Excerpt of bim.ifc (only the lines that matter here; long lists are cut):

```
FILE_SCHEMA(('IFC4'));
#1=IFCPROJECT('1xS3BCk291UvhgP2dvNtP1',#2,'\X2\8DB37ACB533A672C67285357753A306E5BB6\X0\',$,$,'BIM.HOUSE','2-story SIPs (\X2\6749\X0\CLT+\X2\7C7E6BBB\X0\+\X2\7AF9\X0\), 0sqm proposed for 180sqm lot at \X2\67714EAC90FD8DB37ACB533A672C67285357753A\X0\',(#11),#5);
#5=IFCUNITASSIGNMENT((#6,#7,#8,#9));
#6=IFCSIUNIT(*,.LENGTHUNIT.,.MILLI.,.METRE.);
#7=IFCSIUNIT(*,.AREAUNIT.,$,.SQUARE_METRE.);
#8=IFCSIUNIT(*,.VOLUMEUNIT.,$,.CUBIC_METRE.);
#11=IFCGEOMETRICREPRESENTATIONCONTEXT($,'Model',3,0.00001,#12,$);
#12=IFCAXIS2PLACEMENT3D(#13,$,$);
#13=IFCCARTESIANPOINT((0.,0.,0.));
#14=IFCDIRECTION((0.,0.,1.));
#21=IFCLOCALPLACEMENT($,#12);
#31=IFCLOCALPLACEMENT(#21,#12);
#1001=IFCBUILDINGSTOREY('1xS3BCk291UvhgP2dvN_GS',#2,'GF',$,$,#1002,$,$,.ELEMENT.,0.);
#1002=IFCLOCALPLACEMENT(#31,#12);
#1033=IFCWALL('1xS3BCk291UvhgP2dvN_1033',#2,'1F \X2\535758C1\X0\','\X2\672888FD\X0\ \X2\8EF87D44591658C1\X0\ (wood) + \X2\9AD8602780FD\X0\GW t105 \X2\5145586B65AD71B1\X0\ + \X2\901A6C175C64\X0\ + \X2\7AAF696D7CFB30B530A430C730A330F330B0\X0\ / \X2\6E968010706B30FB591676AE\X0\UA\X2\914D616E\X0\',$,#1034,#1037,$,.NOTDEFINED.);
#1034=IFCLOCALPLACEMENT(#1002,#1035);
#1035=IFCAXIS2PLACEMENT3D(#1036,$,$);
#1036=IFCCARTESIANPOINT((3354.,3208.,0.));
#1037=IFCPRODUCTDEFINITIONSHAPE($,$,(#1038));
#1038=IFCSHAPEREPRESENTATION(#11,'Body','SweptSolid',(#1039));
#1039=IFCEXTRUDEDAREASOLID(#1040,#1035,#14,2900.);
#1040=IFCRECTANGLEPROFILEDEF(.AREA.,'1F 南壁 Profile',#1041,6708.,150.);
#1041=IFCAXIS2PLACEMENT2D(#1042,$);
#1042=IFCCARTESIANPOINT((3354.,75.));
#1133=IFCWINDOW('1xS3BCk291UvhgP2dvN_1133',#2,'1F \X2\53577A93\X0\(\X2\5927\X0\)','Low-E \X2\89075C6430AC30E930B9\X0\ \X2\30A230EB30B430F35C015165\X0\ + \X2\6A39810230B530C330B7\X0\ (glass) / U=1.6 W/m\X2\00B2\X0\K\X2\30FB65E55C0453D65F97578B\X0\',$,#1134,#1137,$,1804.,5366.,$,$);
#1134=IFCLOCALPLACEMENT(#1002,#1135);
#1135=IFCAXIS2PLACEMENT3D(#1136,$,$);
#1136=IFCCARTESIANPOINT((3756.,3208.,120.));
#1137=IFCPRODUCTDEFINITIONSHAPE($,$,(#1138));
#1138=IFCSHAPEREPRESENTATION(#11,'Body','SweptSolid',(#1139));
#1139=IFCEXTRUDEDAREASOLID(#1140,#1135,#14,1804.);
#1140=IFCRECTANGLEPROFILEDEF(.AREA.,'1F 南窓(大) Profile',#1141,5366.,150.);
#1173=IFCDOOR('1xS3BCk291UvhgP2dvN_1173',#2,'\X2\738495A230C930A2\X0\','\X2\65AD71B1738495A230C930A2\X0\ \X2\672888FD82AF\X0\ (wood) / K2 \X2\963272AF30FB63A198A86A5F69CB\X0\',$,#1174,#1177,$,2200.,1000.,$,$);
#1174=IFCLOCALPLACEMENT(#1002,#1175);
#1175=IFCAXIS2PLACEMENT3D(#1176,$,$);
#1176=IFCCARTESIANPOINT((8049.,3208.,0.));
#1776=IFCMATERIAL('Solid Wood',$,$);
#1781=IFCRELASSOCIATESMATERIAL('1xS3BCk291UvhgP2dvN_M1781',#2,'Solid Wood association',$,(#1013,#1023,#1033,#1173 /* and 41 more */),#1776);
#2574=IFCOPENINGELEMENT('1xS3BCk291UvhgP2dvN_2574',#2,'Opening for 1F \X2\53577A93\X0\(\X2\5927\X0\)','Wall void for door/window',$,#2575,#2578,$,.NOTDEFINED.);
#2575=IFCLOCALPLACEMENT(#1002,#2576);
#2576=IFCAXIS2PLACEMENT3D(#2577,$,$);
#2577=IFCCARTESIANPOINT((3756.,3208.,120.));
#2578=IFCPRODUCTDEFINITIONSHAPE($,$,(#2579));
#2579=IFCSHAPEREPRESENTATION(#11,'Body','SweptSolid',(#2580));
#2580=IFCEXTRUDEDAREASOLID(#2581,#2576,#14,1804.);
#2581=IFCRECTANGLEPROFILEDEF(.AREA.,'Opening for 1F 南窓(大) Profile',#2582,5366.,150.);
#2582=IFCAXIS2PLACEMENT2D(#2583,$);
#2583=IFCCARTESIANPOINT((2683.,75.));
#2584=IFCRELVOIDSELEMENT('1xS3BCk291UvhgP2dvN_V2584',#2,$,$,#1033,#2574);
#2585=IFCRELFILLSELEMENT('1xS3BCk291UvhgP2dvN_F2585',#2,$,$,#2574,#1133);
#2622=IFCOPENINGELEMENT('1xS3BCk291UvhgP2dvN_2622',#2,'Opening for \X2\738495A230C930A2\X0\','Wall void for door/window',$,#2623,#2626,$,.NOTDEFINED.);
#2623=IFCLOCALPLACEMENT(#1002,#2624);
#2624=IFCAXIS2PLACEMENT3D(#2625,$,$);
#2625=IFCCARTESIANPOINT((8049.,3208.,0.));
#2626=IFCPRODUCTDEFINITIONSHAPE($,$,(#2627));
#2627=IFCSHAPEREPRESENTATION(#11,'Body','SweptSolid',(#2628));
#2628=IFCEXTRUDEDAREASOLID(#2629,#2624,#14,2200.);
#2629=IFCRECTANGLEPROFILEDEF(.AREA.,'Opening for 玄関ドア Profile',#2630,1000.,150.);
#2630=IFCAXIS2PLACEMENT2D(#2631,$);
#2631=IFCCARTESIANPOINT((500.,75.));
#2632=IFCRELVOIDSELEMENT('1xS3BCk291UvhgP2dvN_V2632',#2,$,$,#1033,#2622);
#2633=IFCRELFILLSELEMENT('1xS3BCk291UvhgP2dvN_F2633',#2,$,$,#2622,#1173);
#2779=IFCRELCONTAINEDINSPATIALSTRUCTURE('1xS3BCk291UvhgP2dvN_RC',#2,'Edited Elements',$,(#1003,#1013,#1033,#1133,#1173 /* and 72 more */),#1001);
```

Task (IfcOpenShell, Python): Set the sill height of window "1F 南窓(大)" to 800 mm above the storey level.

```python
import numpy as np
import ifcopenshell
import ifcopenshell.api.geometry
import ifcopenshell.geom
import ifcopenshell.util.element
import ifcopenshell.util.placement
import ifcopenshell.util.shape
import ifcopenshell.util.unit

model = ifcopenshell.open("bim.ifc")
unit_scale = ifcopenshell.util.unit.calculate_unit_scale(model)

window = model.by_guid("1xS3BCk291UvhgP2dvN_1133")
opening = window.FillsVoids[0].RelatingOpeningElement
storey = ifcopenshell.util.element.get_container(window, ifc_class="IfcBuildingStorey")
level = ifcopenshell.util.placement.get_local_placement(storey.ObjectPlacement)[2, 3]

# The opening's origin need not be at the sill, so measure its lowest point.
shape = ifcopenshell.geom.create_shape(ifcopenshell.geom.settings(), opening)
bottom = ifcopenshell.util.shape.get_shape_bottom_elevation(shape, shape.geometry) / unit_scale
dz = level + 0.8 / unit_scale - bottom

shift = np.array([0.0, 0.0, dz])
# The window is not placed relative to its opening, so move both.
for product in (opening, window):
    matrix = ifcopenshell.util.placement.get_local_placement(product.ObjectPlacement)
    matrix[:3, 3] += shift
    ifcopenshell.api.geometry.edit_object_placement(model, product=product, matrix=matrix, is_si=False)

print(f"moved by {dz * unit_scale:+.3f} m")

model.write("bim_v2.ifc")
```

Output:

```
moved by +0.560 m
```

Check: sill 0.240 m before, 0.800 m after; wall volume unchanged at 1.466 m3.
